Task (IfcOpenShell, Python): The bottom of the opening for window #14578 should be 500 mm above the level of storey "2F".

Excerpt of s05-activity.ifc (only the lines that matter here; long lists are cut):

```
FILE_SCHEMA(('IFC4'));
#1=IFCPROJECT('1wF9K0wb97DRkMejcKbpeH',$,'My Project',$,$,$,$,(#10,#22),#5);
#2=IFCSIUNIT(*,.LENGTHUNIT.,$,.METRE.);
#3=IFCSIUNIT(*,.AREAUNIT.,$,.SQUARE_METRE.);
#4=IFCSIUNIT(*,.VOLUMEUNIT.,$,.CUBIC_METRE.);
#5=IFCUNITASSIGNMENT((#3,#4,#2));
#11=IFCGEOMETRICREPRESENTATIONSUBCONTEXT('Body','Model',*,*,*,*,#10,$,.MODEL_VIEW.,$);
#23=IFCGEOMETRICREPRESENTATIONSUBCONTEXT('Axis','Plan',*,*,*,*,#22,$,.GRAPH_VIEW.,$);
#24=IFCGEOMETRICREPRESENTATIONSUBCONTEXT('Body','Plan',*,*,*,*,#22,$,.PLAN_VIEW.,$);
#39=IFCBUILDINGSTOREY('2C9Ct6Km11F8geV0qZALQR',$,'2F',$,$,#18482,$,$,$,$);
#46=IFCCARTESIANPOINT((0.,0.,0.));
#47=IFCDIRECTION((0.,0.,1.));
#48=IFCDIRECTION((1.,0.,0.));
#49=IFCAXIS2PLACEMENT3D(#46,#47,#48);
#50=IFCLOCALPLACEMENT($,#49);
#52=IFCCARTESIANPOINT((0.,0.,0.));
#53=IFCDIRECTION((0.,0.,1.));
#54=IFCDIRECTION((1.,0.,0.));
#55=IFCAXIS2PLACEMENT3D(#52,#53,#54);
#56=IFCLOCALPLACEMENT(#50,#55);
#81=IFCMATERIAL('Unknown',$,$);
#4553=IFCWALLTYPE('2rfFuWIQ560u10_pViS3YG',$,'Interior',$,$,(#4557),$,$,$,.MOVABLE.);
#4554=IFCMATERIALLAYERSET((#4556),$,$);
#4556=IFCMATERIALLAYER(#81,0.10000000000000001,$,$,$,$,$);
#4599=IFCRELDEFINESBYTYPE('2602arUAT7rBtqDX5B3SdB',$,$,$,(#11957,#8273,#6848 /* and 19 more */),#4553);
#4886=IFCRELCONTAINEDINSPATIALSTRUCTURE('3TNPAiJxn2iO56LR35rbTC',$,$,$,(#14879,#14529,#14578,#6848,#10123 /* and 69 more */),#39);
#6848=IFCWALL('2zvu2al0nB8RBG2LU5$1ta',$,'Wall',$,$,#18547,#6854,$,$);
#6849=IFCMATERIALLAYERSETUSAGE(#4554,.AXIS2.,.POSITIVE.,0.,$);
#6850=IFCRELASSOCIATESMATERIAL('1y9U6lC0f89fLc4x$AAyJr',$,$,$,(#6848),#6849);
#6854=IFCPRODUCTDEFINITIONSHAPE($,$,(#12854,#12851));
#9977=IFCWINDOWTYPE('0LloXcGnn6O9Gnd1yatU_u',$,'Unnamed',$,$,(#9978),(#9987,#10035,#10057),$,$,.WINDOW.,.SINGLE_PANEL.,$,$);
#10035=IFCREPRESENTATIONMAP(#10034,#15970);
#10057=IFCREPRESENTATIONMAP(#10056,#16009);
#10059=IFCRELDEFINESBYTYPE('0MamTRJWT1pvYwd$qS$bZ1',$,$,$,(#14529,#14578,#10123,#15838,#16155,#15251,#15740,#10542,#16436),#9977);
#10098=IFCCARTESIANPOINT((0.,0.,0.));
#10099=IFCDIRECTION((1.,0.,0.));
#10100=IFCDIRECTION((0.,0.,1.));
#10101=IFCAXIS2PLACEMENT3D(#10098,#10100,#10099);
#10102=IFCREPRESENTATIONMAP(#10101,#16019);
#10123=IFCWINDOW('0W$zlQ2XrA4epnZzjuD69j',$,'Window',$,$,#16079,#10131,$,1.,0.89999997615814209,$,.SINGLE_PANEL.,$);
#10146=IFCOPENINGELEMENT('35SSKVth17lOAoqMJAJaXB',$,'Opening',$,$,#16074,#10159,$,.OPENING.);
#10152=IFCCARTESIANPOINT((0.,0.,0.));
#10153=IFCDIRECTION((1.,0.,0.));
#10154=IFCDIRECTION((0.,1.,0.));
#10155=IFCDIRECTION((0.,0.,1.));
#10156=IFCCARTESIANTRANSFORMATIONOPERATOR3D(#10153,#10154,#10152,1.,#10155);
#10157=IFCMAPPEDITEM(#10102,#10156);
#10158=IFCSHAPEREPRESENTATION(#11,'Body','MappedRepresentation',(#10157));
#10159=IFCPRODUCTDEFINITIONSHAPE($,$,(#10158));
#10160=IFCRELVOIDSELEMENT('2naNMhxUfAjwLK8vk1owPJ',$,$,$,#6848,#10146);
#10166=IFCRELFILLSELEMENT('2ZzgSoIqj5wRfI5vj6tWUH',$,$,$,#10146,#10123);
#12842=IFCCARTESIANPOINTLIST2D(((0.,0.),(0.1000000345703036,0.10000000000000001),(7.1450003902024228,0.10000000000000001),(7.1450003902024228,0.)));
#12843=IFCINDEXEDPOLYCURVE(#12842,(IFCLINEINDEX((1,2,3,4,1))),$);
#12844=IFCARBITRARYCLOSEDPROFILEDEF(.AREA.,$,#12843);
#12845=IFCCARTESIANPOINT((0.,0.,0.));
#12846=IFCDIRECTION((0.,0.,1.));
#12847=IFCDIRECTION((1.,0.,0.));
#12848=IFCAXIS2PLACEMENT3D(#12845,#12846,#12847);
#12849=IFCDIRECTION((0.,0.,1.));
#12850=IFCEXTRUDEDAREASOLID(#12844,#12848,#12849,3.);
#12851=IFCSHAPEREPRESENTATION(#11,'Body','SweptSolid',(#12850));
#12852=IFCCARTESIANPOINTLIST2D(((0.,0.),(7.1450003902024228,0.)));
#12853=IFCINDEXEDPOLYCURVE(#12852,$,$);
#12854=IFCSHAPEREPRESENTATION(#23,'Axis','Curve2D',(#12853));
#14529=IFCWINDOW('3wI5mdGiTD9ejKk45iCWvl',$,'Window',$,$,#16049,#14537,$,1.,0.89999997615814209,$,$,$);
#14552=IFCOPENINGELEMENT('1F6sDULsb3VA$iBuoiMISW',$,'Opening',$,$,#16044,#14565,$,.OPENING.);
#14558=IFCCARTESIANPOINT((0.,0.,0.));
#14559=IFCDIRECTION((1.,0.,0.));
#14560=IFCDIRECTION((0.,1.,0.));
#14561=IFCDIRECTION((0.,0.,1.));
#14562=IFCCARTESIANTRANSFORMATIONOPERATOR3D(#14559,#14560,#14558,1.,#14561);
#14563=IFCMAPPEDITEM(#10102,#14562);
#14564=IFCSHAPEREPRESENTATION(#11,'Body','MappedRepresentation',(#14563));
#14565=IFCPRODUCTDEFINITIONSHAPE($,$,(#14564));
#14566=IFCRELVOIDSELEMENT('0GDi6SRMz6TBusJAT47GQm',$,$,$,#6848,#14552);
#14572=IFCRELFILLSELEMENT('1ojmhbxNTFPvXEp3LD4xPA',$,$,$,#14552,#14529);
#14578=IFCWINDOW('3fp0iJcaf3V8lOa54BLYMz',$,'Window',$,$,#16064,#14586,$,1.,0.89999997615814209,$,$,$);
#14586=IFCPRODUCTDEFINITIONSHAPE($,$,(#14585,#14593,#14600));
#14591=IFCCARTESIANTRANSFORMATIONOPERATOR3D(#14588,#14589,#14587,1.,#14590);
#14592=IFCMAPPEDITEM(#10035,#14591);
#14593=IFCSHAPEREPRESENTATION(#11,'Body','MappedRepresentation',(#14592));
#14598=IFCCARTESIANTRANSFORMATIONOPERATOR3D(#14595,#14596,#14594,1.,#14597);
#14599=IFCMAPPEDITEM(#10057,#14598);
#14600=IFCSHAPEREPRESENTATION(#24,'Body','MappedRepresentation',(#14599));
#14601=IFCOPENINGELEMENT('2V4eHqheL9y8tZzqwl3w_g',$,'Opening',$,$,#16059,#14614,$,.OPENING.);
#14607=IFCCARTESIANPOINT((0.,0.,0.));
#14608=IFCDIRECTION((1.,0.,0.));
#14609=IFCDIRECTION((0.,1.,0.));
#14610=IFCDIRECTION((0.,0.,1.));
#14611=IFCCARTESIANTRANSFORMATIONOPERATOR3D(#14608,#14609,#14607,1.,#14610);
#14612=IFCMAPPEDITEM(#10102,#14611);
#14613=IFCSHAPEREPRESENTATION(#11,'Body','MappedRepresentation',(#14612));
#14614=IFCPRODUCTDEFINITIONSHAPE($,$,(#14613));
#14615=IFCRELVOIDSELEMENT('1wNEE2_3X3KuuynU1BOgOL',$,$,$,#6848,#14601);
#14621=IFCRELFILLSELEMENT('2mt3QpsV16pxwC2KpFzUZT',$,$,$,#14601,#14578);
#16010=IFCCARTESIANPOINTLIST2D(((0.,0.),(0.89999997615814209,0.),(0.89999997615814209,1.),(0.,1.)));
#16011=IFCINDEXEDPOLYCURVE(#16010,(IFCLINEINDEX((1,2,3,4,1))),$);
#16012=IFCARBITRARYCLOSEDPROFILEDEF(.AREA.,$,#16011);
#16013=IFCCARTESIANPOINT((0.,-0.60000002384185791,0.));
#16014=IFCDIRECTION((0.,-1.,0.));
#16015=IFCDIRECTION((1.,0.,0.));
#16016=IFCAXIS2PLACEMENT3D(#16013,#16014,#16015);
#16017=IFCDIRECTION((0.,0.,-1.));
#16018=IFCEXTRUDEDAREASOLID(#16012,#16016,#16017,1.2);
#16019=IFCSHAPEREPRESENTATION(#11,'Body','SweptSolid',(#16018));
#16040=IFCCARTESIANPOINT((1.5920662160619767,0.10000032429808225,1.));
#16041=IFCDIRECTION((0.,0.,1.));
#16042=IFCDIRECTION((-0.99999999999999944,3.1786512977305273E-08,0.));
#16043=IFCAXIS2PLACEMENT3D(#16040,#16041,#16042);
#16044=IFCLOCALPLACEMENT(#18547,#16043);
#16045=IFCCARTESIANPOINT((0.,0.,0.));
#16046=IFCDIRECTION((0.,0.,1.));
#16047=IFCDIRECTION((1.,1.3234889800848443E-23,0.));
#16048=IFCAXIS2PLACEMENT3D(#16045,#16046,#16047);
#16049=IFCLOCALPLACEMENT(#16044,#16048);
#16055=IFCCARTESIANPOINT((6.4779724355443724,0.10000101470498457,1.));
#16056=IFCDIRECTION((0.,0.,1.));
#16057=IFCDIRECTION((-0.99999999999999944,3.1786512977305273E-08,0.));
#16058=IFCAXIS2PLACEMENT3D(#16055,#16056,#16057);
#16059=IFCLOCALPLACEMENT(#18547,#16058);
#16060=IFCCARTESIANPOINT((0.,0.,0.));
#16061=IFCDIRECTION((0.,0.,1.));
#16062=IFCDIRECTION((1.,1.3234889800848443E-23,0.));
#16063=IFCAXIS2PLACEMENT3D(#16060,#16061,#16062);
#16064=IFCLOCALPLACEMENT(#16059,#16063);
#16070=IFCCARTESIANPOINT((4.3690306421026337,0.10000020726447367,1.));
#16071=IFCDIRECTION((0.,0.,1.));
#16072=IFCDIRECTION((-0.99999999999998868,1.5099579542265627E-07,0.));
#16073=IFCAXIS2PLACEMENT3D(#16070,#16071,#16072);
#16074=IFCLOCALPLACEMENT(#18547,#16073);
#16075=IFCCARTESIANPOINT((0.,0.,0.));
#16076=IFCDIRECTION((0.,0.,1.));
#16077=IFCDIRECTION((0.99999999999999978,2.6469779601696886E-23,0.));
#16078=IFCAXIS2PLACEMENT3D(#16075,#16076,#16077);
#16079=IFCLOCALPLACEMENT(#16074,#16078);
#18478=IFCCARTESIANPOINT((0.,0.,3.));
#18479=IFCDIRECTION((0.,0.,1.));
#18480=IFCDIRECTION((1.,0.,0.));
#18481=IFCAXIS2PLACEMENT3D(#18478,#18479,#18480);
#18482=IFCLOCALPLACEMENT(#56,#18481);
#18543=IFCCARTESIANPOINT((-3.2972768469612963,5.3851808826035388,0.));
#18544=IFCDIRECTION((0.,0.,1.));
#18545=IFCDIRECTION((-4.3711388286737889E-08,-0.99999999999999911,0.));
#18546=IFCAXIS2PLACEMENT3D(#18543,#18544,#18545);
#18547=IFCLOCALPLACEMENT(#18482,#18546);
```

```python
import numpy as np
import ifcopenshell
import ifcopenshell.api.geometry
import ifcopenshell.geom
import ifcopenshell.util.element
import ifcopenshell.util.placement
import ifcopenshell.util.shape
import ifcopenshell.util.unit

model = ifcopenshell.open("s05-activity.ifc")
unit_scale = ifcopenshell.util.unit.calculate_unit_scale(model)

window = model.by_guid("3fp0iJcaf3V8lOa54BLYMz")
opening = window.FillsVoids[0].RelatingOpeningElement
storey = ifcopenshell.util.element.get_container(window, ifc_class="IfcBuildingStorey")
level = ifcopenshell.util.placement.get_local_placement(storey.ObjectPlacement)[2, 3]

# The opening's origin need not be at the sill, so measure its lowest point.
shape = ifcopenshell.geom.create_shape(ifcopenshell.geom.settings(), opening)
bottom = ifcopenshell.util.shape.get_shape_bottom_elevation(shape, shape.geometry) / unit_scale
dz = level + 0.5 / unit_scale - bottom

shift = np.array([0.0, 0.0, dz])
# The window is placed relative to its opening, so it follows when the opening moves.
matrix = ifcopenshell.util.placement.get_local_placement(opening.ObjectPlacement)
matrix[:3, 3] += shift
ifcopenshell.api.geometry.edit_object_placement(
    model, product=opening, matrix=matrix, is_si=False, should_transform_children=True
)

print(f"moved by {dz * unit_scale:+.3f} m")

model.write("s05-activity_updated.ifc")
```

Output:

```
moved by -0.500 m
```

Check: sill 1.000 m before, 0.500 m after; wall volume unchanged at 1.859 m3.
